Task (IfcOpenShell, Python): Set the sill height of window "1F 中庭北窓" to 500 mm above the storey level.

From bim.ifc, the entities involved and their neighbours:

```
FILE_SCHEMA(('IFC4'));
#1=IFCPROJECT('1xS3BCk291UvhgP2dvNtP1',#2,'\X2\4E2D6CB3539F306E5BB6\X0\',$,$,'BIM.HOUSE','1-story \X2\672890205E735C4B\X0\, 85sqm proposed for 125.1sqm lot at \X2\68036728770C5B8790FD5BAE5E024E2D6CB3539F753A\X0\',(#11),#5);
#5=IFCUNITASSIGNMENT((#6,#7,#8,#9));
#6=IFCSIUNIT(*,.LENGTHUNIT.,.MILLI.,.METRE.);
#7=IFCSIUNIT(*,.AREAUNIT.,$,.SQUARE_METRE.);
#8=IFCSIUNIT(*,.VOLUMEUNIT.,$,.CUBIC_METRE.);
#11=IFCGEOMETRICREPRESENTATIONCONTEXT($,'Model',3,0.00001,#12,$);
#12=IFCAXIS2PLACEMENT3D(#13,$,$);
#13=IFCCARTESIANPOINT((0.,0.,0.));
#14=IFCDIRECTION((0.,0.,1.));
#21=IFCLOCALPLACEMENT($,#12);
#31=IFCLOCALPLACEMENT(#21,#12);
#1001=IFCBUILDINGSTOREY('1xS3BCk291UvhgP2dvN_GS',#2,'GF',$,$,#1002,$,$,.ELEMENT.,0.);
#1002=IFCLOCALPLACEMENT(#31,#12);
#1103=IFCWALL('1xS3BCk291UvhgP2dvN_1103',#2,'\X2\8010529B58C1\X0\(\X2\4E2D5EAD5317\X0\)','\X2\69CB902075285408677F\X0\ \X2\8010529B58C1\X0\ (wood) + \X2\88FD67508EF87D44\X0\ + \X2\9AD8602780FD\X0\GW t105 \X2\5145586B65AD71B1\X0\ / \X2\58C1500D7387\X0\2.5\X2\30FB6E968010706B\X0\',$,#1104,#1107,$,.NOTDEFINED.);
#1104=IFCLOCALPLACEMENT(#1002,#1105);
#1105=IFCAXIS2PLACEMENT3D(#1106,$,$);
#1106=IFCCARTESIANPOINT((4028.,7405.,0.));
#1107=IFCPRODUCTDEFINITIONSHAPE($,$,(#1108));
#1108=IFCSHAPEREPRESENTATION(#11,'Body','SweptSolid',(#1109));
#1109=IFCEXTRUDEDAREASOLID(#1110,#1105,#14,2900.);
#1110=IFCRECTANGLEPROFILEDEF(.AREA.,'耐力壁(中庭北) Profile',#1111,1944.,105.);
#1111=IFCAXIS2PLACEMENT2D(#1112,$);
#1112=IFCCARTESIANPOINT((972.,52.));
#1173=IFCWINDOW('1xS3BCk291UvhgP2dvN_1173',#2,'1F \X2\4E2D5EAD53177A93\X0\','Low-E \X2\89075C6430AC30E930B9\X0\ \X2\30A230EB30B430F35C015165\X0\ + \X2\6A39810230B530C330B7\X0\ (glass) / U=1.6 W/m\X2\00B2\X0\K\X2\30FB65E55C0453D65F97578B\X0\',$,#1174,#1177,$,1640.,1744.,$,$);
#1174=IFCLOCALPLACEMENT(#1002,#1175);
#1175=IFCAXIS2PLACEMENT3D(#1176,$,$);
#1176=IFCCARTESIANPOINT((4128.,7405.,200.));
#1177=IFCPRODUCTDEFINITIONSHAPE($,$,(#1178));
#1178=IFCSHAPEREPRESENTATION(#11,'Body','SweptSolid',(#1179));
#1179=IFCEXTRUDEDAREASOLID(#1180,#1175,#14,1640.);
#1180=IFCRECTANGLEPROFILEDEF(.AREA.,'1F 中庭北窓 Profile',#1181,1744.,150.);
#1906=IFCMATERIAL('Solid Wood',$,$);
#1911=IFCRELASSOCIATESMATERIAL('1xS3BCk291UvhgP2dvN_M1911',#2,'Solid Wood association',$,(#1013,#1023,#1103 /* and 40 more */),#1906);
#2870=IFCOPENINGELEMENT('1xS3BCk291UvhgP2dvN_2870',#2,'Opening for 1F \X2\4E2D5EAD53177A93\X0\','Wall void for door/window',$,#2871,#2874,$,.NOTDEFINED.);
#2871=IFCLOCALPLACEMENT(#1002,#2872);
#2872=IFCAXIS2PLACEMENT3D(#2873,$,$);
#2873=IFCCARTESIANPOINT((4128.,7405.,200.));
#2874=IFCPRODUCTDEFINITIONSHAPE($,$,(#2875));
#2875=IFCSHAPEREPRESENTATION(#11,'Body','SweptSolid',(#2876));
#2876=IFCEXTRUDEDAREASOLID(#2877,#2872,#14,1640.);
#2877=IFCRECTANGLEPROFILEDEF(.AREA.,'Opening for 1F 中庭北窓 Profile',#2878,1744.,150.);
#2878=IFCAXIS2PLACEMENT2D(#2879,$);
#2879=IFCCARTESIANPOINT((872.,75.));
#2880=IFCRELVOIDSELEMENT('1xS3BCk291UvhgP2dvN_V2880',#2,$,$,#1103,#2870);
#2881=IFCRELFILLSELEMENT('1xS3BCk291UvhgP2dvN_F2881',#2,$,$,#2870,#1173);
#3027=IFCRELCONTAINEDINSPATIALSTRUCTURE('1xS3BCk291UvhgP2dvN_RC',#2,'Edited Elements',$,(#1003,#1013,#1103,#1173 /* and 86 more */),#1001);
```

```python
import numpy as np
import ifcopenshell
import ifcopenshell.api.geometry
import ifcopenshell.geom
import ifcopenshell.util.element
import ifcopenshell.util.placement
import ifcopenshell.util.shape
import ifcopenshell.util.unit

model = ifcopenshell.open("bim.ifc")
unit_scale = ifcopenshell.util.unit.calculate_unit_scale(model)

window = model.by_id(1173)
opening = window.FillsVoids[0].RelatingOpeningElement
storey = ifcopenshell.util.element.get_container(window, ifc_class="IfcBuildingStorey")
level = ifcopenshell.util.placement.get_local_placement(storey.ObjectPlacement)[2, 3]

# The opening's origin need not be at the sill, so measure its lowest point.
shape = ifcopenshell.geom.create_shape(ifcopenshell.geom.settings(), opening)
bottom = ifcopenshell.util.shape.get_shape_bottom_elevation(shape, shape.geometry) / unit_scale
dz = level + 0.5 / unit_scale - bottom

shift = np.array([0.0, 0.0, dz])
# The window is not placed relative to its opening, so move both.
for product in (opening, window):
    matrix = ifcopenshell.util.placement.get_local_placement(product.ObjectPlacement)
    matrix[:3, 3] += shift
    ifcopenshell.api.geometry.edit_object_placement(model, product=product, matrix=matrix, is_si=False)

print(f"moved by {dz * unit_scale:+.3f} m")

model.write("bim_rev.ifc")
```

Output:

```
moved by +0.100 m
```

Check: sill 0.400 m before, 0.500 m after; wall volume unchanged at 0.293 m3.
